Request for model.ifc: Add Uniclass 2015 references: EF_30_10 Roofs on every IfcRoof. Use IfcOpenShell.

First a look at what the model holds.

```python
import ifcopenshell

model = ifcopenshell.open("model.ifc")
print(model.schema)
print("classifications:", [c.Name for c in model.by_type("IfcClassification")])
for ifc_class in ("IfcDoor", "IfcRoof", "IfcStair", "IfcWall", "IfcWindow"):
    print(ifc_class, len(model.by_type(ifc_class)))
```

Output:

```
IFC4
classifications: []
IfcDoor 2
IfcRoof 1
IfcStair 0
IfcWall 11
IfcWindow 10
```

```python
import ifcopenshell
import ifcopenshell.api.classification

model = ifcopenshell.open("model.ifc")

system = ifcopenshell.api.classification.add_classification(model, classification="Uniclass 2015")

codes = {
    "IfcRoof": ("EF_30_10", "Roofs"),
}
for ifc_class, (code, name) in codes.items():
    products = model.by_type(ifc_class)
    ifcopenshell.api.classification.add_reference(
        model, products=products, classification=system, identification=code, name=name
    )
    print(code, len(products))

model.write("model_edited.ifc")
```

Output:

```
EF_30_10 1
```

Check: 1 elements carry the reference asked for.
